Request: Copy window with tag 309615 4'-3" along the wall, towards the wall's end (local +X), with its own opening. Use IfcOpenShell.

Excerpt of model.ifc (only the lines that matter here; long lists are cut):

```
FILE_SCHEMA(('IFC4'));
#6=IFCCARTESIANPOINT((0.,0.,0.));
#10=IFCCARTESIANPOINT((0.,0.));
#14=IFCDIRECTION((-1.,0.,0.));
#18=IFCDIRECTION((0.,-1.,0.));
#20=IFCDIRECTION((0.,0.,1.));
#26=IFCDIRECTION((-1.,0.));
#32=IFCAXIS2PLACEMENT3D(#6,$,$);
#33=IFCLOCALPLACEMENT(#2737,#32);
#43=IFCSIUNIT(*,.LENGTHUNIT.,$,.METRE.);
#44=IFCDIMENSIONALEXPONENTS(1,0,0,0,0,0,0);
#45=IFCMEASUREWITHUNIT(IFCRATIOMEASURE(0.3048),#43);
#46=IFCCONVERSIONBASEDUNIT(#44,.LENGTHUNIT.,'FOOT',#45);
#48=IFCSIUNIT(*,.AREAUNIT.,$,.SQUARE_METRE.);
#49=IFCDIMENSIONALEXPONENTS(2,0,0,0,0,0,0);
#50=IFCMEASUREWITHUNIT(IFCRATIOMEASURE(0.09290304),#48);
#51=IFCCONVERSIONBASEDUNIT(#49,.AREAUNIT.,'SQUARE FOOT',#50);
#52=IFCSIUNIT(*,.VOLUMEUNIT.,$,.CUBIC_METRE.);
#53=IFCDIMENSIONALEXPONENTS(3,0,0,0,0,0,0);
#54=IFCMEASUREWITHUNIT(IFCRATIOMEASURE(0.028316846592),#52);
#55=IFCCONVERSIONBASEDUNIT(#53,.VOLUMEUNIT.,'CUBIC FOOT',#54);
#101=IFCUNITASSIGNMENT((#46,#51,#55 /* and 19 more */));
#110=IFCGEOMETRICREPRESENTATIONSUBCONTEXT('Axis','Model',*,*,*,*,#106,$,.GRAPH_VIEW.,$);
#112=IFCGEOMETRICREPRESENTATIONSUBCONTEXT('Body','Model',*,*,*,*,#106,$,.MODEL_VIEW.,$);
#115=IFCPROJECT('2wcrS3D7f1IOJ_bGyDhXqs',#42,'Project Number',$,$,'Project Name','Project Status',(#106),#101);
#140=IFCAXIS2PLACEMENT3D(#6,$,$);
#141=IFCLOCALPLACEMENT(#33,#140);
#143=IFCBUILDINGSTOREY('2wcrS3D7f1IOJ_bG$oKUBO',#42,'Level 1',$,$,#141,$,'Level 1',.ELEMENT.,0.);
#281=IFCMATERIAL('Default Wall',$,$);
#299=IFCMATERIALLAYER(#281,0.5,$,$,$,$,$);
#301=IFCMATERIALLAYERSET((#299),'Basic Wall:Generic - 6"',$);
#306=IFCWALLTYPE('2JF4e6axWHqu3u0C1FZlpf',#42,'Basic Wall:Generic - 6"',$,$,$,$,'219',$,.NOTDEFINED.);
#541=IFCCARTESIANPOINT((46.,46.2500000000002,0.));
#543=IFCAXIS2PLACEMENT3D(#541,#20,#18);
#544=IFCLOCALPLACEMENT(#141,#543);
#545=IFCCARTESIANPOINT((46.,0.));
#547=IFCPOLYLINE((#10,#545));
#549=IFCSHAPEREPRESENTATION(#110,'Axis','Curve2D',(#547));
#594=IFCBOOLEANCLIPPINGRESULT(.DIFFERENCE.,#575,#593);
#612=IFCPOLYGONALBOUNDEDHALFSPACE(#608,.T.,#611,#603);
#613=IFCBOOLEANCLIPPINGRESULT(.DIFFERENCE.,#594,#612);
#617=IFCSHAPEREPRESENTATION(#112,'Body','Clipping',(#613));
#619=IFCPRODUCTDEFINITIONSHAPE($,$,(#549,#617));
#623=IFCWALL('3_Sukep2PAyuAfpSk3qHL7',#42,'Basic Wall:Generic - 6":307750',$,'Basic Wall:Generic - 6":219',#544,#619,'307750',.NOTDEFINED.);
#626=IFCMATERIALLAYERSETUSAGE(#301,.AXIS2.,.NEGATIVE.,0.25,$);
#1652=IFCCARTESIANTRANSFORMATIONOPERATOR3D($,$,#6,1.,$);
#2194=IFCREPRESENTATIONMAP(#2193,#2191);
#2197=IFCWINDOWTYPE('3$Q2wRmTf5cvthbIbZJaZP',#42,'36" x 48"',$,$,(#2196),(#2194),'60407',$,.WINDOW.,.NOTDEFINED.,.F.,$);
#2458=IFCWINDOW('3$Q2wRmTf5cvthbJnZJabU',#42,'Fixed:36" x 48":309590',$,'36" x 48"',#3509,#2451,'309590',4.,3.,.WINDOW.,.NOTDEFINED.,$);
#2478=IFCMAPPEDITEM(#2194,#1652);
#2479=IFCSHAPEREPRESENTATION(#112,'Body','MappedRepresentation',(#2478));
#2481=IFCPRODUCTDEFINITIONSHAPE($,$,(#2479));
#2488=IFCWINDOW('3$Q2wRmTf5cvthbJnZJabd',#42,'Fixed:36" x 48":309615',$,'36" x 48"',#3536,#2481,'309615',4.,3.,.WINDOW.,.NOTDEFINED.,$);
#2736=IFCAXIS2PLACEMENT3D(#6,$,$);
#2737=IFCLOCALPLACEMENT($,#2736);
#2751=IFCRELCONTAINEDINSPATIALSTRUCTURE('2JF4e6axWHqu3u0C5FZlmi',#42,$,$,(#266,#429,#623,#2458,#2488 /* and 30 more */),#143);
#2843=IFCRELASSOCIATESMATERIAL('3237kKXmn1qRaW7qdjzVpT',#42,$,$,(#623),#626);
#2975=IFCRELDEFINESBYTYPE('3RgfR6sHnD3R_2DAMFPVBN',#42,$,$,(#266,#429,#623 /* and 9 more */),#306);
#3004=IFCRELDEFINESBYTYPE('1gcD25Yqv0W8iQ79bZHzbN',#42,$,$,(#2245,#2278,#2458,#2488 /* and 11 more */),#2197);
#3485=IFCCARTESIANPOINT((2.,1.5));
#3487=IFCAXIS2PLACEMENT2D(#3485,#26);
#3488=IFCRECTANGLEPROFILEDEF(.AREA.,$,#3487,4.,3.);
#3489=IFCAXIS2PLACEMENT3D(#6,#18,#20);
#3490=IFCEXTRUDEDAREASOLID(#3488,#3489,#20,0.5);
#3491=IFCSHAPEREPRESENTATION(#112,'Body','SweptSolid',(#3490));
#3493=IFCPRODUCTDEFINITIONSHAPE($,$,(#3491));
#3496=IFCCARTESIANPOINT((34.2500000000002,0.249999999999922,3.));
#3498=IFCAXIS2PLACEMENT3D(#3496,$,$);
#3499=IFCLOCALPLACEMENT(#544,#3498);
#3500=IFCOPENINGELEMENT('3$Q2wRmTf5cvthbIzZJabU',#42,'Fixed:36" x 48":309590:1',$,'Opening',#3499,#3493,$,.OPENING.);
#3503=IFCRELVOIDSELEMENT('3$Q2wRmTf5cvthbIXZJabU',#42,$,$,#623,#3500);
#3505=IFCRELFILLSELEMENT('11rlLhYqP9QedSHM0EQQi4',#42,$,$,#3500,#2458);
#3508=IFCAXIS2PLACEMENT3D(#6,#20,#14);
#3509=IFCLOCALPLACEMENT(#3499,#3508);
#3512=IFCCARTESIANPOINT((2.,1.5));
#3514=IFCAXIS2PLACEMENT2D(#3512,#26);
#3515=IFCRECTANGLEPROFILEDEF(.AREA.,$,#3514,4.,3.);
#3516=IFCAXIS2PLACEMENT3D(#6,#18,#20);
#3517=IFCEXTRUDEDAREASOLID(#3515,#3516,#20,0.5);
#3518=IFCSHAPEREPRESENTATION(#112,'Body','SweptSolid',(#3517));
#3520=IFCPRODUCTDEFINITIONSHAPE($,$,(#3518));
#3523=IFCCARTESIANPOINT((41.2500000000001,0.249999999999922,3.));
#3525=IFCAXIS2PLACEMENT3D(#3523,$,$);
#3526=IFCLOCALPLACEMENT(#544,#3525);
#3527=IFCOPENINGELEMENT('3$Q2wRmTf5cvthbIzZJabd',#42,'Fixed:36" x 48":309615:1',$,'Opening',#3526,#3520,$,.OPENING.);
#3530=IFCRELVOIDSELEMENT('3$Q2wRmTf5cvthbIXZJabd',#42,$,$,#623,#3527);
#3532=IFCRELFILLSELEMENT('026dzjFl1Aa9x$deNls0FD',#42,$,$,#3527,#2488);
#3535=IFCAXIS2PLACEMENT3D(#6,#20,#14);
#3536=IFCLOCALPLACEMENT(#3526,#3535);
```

```python
import ifcopenshell
import ifcopenshell.api.feature
import ifcopenshell.api.geometry
import ifcopenshell.api.root
import ifcopenshell.geom
import ifcopenshell.util.element
import ifcopenshell.util.placement
import ifcopenshell.util.shape
import ifcopenshell.util.unit

model = ifcopenshell.open("model.ifc")
unit_scale = ifcopenshell.util.unit.calculate_unit_scale(model)
settings = ifcopenshell.geom.settings()


def volume(element):
    """Net volume in cubic metres, openings subtracted."""
    shape = ifcopenshell.geom.create_shape(settings, element)
    return ifcopenshell.util.shape.get_volume(shape.geometry)


def reuse_history(source, copy):
    """copy_class also copies each property set's owner history, people and application; keep the originals."""
    for rel in copy.IsDefinedBy:
        if rel.is_a("IfcRelDefinesByProperties") and (history := rel.RelatingPropertyDefinition.OwnerHistory):
            rel.RelatingPropertyDefinition.OwnerHistory = source.OwnerHistory
            ifcopenshell.util.element.remove_deep2(model, history)


window = model.by_guid("3$Q2wRmTf5cvthbJnZJabd")
opening = window.FillsVoids[0].RelatingOpeningElement
wall = opening.VoidsElements[0].RelatingBuildingElement
before = volume(wall)
shift = ifcopenshell.util.placement.get_local_placement(wall.ObjectPlacement)[:3, 0] * 51 * 0.0254 / unit_scale

# copy_class copies the void relationship, type, container and properties, but no geometry.
new_opening = ifcopenshell.api.root.copy_class(model, product=opening)
new_opening.Representation = ifcopenshell.util.element.copy_deep(
    model, opening.Representation, exclude=["IfcGeometricRepresentationContext", "IfcRepresentationMap"]
)
new_opening.Name = 'Fixed:36" x 48"'
new_window = ifcopenshell.api.root.copy_class(model, product=window)
new_window.Representation = ifcopenshell.util.element.copy_deep(
    model, window.Representation, exclude=["IfcGeometricRepresentationContext", "IfcRepresentationMap"]
)
new_window.Name = 'Fixed:36" x 48"'
new_window.Tag = None
reuse_history(window, new_window)
ifcopenshell.api.feature.add_filling(model, opening=new_opening, element=new_window)

for old, new in ((opening, new_opening), (window, new_window)):
    matrix = ifcopenshell.util.placement.get_local_placement(old.ObjectPlacement)
    matrix[:3, 3] += shift
    ifcopenshell.api.geometry.edit_object_placement(model, product=new, matrix=matrix, is_si=False)

after = volume(wall)

print(f"wall volume {before:.3f} -> {after:.3f} m3")

model.write("model_updated.ifc")
```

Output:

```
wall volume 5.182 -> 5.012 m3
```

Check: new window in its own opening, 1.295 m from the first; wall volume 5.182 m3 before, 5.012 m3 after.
